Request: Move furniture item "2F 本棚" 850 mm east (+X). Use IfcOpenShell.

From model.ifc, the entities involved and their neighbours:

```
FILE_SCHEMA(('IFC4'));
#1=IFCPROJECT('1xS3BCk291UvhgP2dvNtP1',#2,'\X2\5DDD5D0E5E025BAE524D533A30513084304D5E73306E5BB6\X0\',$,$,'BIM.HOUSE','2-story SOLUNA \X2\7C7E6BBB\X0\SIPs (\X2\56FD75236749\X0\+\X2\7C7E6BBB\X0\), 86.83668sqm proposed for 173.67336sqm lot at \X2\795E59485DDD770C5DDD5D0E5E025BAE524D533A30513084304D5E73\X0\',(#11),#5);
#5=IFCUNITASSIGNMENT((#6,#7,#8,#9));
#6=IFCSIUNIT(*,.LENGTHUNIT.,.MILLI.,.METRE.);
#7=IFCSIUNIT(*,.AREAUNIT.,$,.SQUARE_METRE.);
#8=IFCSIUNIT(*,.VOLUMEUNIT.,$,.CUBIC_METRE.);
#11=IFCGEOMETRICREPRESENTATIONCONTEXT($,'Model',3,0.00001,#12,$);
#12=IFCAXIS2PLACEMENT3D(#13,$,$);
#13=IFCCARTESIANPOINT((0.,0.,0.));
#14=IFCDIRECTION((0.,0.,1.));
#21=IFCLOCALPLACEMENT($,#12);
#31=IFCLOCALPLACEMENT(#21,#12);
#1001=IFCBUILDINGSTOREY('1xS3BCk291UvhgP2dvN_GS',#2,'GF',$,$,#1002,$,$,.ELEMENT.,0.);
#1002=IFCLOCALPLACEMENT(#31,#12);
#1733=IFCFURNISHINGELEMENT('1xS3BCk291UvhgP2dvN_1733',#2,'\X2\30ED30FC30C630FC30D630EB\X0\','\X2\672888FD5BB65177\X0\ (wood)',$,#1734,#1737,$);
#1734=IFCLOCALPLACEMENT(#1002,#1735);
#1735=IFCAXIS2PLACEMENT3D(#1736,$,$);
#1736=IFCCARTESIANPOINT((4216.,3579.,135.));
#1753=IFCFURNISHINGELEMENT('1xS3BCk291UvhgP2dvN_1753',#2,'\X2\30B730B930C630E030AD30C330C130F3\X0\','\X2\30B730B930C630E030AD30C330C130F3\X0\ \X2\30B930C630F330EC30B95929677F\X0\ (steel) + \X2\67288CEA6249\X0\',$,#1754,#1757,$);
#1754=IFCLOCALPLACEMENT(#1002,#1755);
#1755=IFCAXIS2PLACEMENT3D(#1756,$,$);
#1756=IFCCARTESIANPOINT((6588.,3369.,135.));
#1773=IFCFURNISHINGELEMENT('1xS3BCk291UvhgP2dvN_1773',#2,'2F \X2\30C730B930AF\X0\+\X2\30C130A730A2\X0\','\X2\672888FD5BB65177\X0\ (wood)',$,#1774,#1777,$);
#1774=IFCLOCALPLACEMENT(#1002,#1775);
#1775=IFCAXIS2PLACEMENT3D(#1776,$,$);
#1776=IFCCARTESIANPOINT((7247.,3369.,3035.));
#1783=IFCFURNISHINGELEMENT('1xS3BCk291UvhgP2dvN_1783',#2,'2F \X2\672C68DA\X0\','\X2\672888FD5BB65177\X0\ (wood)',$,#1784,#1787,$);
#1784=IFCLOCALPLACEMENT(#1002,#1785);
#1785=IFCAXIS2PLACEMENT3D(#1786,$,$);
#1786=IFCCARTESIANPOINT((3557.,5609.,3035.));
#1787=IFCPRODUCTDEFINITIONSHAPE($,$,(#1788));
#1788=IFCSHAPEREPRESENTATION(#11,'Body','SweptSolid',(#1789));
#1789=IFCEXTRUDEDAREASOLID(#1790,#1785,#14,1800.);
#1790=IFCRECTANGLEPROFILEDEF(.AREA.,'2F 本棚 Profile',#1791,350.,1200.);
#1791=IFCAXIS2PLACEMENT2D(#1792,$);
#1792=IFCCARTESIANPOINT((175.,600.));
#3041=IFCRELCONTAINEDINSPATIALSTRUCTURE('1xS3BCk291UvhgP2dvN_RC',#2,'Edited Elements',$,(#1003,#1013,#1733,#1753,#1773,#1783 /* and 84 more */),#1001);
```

```python
import ifcopenshell
import ifcopenshell.api.geometry
import ifcopenshell.util.placement
import ifcopenshell.util.unit

model = ifcopenshell.open("model.ifc")
unit_scale = ifcopenshell.util.unit.calculate_unit_scale(model)

item = model.by_guid("1xS3BCk291UvhgP2dvN_1783")
matrix = ifcopenshell.util.placement.get_local_placement(item.ObjectPlacement)
matrix[0, 3] += 0.85 / unit_scale
ifcopenshell.api.geometry.edit_object_placement(model, product=item, matrix=matrix, is_si=False)

print(ifcopenshell.util.placement.get_local_placement(item.ObjectPlacement).round(3) + 0.0)

model.write("model-out.ifc")
```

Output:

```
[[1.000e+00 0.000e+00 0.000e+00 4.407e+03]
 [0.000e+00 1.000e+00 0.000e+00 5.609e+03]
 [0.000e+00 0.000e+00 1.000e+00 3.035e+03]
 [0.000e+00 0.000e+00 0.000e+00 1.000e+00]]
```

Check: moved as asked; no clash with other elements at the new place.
